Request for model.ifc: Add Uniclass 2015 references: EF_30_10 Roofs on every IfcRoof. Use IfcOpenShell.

First a look at what the model holds.

```python
import ifcopenshell

model = ifcopenshell.open("model.ifc")
print(model.schema)
print("classifications:", [c.Name for c in model.by_type("IfcClassification")])
for ifc_class in ("IfcDoor", "IfcRoof", "IfcStair", "IfcWall", "IfcWindow"):
    print(ifc_class, len(model.by_type(ifc_class)))
```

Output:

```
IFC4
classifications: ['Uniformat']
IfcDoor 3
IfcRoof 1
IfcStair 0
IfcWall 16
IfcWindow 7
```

```python
import ifcopenshell
import ifcopenshell.api.classification

model = ifcopenshell.open("model.ifc")

system = ifcopenshell.api.classification.add_classification(model, classification="Uniclass 2015")

codes = {
    "IfcRoof": ("EF_30_10", "Roofs"),
}
for ifc_class, (code, name) in codes.items():
    products = model.by_type(ifc_class)
    ifcopenshell.api.classification.add_reference(
        model, products=products, classification=system, identification=code, name=name
    )
    print(code, len(products))

model.write("model_edited.ifc")
```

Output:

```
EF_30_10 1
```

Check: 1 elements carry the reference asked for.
